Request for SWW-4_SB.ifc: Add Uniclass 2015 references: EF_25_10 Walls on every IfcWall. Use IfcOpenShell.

First a look at what the model holds.

```python
import ifcopenshell

model = ifcopenshell.open("SWW-4_SB.ifc")
print(model.schema)
print("classifications:", [c.Name for c in model.by_type("IfcClassification")])
for ifc_class in ("IfcDoor", "IfcRoof", "IfcStair", "IfcWall", "IfcWindow"):
    print(ifc_class, len(model.by_type(ifc_class)))
```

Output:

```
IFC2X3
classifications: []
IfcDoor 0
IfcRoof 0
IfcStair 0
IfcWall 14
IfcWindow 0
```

```python
import ifcopenshell
import ifcopenshell.api.classification

model = ifcopenshell.open("SWW-4_SB.ifc")

# IFC2X3 requires Source and Edition and has no link from the project to the system.
system = model.create_entity("IfcClassification", Source="NBS", Edition="2015", Name="Uniclass 2015")

codes = {
    "IfcWall": ("EF_25_10", "Walls"),
}
for ifc_class, (code, name) in codes.items():
    products = model.by_type(ifc_class)
    ifcopenshell.api.classification.add_reference(
        model, products=products, classification=system, identification=code, name=name
    )
    print(code, len(products))

model.write("SWW-4_SB_updated.ifc")
```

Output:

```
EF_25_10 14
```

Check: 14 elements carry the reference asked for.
